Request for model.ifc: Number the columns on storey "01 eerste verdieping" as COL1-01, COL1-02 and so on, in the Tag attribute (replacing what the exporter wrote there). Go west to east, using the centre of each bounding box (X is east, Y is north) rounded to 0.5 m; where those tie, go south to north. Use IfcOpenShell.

First a look at what the model holds.

```python
import ifcopenshell
import ifcopenshell.util.element
import ifcopenshell.util.placement

model = ifcopenshell.open("model.ifc")
print(model.schema)
storey = next(s for s in model.by_type("IfcBuildingStorey") if s.Name == "01 eerste verdieping")
columns = [e for e in ifcopenshell.util.element.get_decomposition(storey) if e.is_a("IfcColumn")]
for e in sorted(columns, key=lambda e: e.id()):
    origin = ifcopenshell.util.placement.get_local_placement(e.ObjectPlacement)[:3, 3]
    print(e.id(), e.Tag, e.Name, origin.round(2) + 0.0, sep=" | ")
```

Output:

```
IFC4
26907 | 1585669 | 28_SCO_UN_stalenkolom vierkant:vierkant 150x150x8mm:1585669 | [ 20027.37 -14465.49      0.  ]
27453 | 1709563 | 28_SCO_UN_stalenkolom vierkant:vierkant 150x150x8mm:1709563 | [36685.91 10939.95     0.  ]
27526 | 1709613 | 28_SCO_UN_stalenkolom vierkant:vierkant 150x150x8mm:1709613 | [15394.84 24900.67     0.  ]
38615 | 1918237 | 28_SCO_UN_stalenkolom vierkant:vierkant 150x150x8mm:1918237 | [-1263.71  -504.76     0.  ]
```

```python
import ifcopenshell
import ifcopenshell.geom
import ifcopenshell.util.element
import ifcopenshell.util.shape

model = ifcopenshell.open("model.ifc")
settings = ifcopenshell.geom.settings()
settings.set("use-world-coords", True)


def centre(element):
    shape = ifcopenshell.geom.create_shape(settings, element)
    return ifcopenshell.util.shape.get_bbox_centroid(shape.geometry)


storey = next(s for s in model.by_type("IfcBuildingStorey") if s.Name == "01 eerste verdieping")
columns = [e for e in ifcopenshell.util.element.get_decomposition(storey) if e.is_a("IfcColumn")]

# Insertion points can sit at a corner or the storey origin, so sort by the geometry (in metres).
centres = {e: centre(e) for e in columns}
columns.sort(key=lambda e: (round(centres[e][0] / 0.5), centres[e][1]))

for i, e in enumerate(columns, start=1):
    number = f"COL1-{i:02d}"
    e.Tag = number
    print(e.id(), number)

model.write("model_edited.ifc")
```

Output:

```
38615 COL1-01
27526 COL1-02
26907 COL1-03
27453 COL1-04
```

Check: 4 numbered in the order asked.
